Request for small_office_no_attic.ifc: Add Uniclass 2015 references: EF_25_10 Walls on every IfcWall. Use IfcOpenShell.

First a look at what the model holds.

```python
import ifcopenshell

model = ifcopenshell.open("small_office_no_attic.ifc")
print(model.schema)
print("classifications:", [c.Name for c in model.by_type("IfcClassification")])
for ifc_class in ("IfcDoor", "IfcRoof", "IfcStair", "IfcWall", "IfcWindow"):
    print(ifc_class, len(model.by_type(ifc_class)))
```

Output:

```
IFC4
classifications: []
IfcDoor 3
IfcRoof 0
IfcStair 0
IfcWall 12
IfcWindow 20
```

```python
import ifcopenshell
import ifcopenshell.api.classification

model = ifcopenshell.open("small_office_no_attic.ifc")

system = ifcopenshell.api.classification.add_classification(model, classification="Uniclass 2015")

codes = {
    "IfcWall": ("EF_25_10", "Walls"),
}
for ifc_class, (code, name) in codes.items():
    products = model.by_type(ifc_class)
    ifcopenshell.api.classification.add_reference(
        model, products=products, classification=system, identification=code, name=name
    )
    print(code, len(products))

model.write("small_office_no_attic-out.ifc")
```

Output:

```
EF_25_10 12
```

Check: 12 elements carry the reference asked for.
